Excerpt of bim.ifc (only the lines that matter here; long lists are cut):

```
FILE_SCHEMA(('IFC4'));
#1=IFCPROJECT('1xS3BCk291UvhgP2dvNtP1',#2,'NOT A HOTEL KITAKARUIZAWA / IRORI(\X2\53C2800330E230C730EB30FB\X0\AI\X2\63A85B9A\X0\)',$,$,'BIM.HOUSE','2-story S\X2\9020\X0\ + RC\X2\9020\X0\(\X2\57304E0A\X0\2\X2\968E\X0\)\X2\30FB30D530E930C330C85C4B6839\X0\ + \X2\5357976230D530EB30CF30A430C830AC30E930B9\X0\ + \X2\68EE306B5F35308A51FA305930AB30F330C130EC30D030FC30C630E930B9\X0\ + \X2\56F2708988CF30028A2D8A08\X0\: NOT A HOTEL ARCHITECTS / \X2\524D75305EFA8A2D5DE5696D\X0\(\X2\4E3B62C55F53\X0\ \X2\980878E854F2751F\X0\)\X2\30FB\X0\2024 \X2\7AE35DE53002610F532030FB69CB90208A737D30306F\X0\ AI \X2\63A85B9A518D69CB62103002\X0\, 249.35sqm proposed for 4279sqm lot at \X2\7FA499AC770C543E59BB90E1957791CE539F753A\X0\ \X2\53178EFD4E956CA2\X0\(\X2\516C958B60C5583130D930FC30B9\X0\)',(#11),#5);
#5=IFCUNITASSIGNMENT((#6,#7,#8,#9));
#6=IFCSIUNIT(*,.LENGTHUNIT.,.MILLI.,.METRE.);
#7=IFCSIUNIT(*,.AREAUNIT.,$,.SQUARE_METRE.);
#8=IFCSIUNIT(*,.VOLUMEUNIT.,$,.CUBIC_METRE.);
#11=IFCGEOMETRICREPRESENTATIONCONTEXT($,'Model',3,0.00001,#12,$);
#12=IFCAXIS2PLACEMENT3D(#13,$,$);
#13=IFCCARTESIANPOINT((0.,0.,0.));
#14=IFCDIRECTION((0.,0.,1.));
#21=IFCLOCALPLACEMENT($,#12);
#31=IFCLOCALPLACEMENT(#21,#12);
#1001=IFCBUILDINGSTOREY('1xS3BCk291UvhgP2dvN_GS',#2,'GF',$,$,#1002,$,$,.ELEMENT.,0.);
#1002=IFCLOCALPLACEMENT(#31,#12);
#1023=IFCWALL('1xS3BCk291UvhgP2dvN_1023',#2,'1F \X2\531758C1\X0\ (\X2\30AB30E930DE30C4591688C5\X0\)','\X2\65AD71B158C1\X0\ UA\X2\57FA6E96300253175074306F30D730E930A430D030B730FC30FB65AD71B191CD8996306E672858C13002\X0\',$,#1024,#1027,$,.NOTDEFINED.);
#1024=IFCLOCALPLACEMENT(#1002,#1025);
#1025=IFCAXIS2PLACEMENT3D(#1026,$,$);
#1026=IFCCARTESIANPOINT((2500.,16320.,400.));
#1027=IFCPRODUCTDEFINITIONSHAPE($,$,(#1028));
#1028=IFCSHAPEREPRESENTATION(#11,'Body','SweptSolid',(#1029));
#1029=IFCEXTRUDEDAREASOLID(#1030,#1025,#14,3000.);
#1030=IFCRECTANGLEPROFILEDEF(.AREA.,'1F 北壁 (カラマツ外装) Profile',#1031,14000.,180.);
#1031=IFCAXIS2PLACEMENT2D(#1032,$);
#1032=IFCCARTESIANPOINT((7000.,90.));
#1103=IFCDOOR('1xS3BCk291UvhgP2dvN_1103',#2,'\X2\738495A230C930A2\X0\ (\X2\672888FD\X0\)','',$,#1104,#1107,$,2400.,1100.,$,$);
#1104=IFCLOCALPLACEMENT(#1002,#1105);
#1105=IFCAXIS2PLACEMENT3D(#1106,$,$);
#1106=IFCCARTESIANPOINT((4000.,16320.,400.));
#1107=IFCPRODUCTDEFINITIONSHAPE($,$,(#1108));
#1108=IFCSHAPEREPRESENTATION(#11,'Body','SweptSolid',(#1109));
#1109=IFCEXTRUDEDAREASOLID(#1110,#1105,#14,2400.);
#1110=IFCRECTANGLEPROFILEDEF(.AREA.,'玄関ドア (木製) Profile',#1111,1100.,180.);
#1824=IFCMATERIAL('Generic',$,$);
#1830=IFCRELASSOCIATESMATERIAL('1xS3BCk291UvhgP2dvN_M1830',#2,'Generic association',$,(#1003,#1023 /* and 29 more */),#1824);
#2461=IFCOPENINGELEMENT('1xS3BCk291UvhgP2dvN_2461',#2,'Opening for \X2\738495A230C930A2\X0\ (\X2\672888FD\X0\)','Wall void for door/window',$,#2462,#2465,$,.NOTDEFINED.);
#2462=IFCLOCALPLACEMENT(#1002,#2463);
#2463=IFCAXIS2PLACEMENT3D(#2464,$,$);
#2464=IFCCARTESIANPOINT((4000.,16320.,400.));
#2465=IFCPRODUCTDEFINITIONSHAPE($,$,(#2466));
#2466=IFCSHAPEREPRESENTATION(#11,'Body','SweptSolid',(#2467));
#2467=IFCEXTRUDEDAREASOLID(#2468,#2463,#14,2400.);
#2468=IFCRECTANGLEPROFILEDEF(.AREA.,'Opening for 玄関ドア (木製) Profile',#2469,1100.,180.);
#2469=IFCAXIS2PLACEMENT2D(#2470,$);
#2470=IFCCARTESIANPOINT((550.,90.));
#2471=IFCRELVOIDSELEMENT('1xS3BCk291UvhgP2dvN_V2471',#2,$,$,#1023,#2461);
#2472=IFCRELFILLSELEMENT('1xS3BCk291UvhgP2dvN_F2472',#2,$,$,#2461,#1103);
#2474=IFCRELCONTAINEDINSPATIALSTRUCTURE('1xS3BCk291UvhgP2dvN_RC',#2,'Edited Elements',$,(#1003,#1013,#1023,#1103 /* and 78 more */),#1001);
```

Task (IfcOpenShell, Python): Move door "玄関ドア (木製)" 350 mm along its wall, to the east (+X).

```python
import ifcopenshell
import ifcopenshell.api.geometry
import ifcopenshell.util.placement
import ifcopenshell.util.unit

model = ifcopenshell.open("bim.ifc")
unit_scale = ifcopenshell.util.unit.calculate_unit_scale(model)

door = model.by_guid("1xS3BCk291UvhgP2dvN_1103")
opening = door.FillsVoids[0].RelatingOpeningElement
wall = opening.VoidsElements[0].RelatingBuildingElement

wall_matrix = ifcopenshell.util.placement.get_local_placement(wall.ObjectPlacement)
shift = wall_matrix[:3, 0] * 0.35 / unit_scale
before = ifcopenshell.util.placement.get_local_placement(door.ObjectPlacement)[:3, 3].copy()

# The door is not placed relative to its opening, so move both.
for product in (opening, door):
    matrix = ifcopenshell.util.placement.get_local_placement(product.ObjectPlacement)
    matrix[:3, 3] += shift
    ifcopenshell.api.geometry.edit_object_placement(model, product=product, matrix=matrix, is_si=False)

after = ifcopenshell.util.placement.get_local_placement(door.ObjectPlacement)[:3, 3]
print("door moved by", (after - before).round(3) + 0.0)

model.write("bim_v2.ifc")
```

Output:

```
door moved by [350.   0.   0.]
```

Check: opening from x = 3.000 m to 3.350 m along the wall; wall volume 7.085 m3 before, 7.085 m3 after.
